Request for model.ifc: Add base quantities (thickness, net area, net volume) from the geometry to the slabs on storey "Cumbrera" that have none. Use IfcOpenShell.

First a look at what the model holds.

```python
import ifcopenshell
import ifcopenshell.util.element
import ifcopenshell.util.unit

model = ifcopenshell.open("model.ifc")
print(model.schema)
for unit_type in ("LENGTHUNIT", "AREAUNIT", "VOLUMEUNIT"):
    print(unit_type, ifcopenshell.util.unit.calculate_unit_scale(model, unit_type))
storey = next(s for s in model.by_type("IfcBuildingStorey") if s.Name == "Cumbrera")
slabs = [e for e in ifcopenshell.util.element.get_decomposition(storey) if e.is_a("IfcSlab")]
for e in sorted(slabs, key=lambda e: e.id()):
    print(e.id(), e.is_a(), e.Name, list(ifcopenshell.util.element.get_psets(e, qtos_only=True)), sep=" | ")
```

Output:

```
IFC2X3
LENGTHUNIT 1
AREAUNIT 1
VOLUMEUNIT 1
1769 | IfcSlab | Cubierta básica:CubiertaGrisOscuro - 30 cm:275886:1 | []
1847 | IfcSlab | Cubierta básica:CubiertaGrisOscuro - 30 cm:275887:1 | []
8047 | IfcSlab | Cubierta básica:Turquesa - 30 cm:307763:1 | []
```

```python
import ifcopenshell
import ifcopenshell.api.pset
import ifcopenshell.geom
import ifcopenshell.util.element
import ifcopenshell.util.shape
import ifcopenshell.util.unit

model = ifcopenshell.open("model.ifc")
unit_scale = ifcopenshell.util.unit.calculate_unit_scale(model)
area_scale = ifcopenshell.util.unit.calculate_unit_scale(model, "AREAUNIT")
volume_scale = ifcopenshell.util.unit.calculate_unit_scale(model, "VOLUMEUNIT")
settings = ifcopenshell.geom.settings()

storey = next(s for s in model.by_type("IfcBuildingStorey") if s.Name == "Cumbrera")
slabs = [e for e in ifcopenshell.util.element.get_decomposition(storey) if e.is_a("IfcSlab")]

for e in sorted(slabs, key=lambda e: e.id()):
    if ifcopenshell.util.element.get_psets(e, qtos_only=True, should_inherit=False):
        continue
    # Geometry comes back in metres, in the element's own axes.
    shape = ifcopenshell.geom.create_shape(settings, e)
    values = {
        "Width": ifcopenshell.util.shape.get_z(shape.geometry) / unit_scale,
        "NetArea": ifcopenshell.util.shape.get_footprint_area(shape.geometry) / area_scale,
        "NetVolume": ifcopenshell.util.shape.get_volume(shape.geometry) / volume_scale,
    }
    qto = ifcopenshell.api.pset.add_qto(model, product=e, name="BaseQuantities")
    ifcopenshell.api.pset.edit_qto(model, qto=qto, properties=values)
    print(e.id(), {k: round(v, 3) for k, v in values.items()})

model.write("model_updated.ifc")
```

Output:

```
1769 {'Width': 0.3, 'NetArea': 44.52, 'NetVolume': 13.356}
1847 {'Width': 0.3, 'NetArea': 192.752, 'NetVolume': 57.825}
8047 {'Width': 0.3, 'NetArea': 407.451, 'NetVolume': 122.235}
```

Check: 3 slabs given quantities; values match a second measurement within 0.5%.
